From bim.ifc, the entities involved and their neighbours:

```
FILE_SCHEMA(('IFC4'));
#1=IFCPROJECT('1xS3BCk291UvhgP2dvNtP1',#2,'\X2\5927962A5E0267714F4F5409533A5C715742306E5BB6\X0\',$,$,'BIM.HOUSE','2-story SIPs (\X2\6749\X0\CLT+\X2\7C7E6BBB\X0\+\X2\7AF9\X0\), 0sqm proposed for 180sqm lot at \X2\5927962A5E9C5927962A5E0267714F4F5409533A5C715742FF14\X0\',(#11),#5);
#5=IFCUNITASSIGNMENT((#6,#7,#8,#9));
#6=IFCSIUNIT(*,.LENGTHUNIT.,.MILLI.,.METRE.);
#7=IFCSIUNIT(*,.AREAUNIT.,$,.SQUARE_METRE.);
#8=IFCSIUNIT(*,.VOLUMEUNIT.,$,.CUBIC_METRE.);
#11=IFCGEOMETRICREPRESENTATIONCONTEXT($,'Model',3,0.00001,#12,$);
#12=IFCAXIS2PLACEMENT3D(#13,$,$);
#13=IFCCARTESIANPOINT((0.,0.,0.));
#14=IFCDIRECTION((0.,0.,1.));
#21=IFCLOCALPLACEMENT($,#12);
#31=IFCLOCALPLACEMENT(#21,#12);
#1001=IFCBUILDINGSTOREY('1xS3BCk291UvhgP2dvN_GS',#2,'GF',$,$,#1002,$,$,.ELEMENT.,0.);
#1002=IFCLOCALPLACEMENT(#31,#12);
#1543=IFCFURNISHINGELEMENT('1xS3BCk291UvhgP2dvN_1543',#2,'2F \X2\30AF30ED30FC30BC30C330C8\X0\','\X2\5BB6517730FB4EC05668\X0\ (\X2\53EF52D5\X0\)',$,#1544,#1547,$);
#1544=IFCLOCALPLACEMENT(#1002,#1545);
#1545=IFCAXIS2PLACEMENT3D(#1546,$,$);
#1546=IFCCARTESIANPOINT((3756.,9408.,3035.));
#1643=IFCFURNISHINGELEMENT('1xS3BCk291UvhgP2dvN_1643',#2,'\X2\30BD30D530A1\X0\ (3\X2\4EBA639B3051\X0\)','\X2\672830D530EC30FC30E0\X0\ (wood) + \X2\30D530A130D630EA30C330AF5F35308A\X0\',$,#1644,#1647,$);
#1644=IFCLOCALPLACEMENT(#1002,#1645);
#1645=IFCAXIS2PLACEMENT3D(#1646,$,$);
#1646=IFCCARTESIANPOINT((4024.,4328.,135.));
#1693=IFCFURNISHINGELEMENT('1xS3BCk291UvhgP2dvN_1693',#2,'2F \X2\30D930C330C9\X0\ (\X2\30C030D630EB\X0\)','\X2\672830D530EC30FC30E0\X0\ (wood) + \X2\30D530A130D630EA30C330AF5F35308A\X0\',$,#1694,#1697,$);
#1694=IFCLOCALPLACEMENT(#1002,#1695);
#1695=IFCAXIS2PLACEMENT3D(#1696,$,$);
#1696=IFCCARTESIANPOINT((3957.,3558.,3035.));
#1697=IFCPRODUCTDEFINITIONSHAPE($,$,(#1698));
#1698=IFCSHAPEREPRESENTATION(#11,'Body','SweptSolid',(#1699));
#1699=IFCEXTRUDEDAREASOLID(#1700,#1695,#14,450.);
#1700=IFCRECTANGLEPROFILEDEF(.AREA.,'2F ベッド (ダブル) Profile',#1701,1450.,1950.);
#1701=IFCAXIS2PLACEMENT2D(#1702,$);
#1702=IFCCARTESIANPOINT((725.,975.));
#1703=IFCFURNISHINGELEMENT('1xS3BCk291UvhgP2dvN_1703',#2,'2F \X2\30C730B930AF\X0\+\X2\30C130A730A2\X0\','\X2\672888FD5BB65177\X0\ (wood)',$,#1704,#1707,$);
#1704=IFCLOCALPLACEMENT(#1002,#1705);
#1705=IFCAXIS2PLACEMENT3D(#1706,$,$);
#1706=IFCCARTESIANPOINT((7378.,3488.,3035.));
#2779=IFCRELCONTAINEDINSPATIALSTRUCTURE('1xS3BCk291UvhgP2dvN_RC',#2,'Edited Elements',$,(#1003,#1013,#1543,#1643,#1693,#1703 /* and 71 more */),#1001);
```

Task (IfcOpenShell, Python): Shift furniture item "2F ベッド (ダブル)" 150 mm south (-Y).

```python
import ifcopenshell
import ifcopenshell.api.geometry
import ifcopenshell.util.placement
import ifcopenshell.util.unit

model = ifcopenshell.open("bim.ifc")
unit_scale = ifcopenshell.util.unit.calculate_unit_scale(model)

item = model.by_guid("1xS3BCk291UvhgP2dvN_1693")
matrix = ifcopenshell.util.placement.get_local_placement(item.ObjectPlacement)
matrix[1, 3] -= 0.15 / unit_scale
ifcopenshell.api.geometry.edit_object_placement(model, product=item, matrix=matrix, is_si=False)

print(ifcopenshell.util.placement.get_local_placement(item.ObjectPlacement).round(3) + 0.0)

model.write("bim_rev.ifc")
```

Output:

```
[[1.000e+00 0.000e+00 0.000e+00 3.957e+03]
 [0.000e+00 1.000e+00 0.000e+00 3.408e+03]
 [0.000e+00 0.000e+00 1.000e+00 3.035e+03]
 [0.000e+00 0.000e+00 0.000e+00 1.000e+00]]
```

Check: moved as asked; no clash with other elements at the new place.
